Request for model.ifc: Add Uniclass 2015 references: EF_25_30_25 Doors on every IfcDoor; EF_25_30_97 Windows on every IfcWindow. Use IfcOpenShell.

First a look at what the model holds.

```python
import ifcopenshell

model = ifcopenshell.open("model.ifc")
print(model.schema)
print("classifications:", [c.Name for c in model.by_type("IfcClassification")])
for ifc_class in ("IfcDoor", "IfcRoof", "IfcStair", "IfcWall", "IfcWindow"):
    print(ifc_class, len(model.by_type(ifc_class)))
```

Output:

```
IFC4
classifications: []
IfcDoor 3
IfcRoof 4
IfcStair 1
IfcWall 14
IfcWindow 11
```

```python
import ifcopenshell
import ifcopenshell.api.classification

model = ifcopenshell.open("model.ifc")

system = ifcopenshell.api.classification.add_classification(model, classification="Uniclass 2015")

codes = {
    "IfcDoor": ("EF_25_30_25", "Doors"),
    "IfcWindow": ("EF_25_30_97", "Windows"),
}
for ifc_class, (code, name) in codes.items():
    products = model.by_type(ifc_class)
    ifcopenshell.api.classification.add_reference(
        model, products=products, classification=system, identification=code, name=name
    )
    print(code, len(products))

model.write("model-out.ifc")
```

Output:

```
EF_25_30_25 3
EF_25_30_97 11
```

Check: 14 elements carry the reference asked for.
